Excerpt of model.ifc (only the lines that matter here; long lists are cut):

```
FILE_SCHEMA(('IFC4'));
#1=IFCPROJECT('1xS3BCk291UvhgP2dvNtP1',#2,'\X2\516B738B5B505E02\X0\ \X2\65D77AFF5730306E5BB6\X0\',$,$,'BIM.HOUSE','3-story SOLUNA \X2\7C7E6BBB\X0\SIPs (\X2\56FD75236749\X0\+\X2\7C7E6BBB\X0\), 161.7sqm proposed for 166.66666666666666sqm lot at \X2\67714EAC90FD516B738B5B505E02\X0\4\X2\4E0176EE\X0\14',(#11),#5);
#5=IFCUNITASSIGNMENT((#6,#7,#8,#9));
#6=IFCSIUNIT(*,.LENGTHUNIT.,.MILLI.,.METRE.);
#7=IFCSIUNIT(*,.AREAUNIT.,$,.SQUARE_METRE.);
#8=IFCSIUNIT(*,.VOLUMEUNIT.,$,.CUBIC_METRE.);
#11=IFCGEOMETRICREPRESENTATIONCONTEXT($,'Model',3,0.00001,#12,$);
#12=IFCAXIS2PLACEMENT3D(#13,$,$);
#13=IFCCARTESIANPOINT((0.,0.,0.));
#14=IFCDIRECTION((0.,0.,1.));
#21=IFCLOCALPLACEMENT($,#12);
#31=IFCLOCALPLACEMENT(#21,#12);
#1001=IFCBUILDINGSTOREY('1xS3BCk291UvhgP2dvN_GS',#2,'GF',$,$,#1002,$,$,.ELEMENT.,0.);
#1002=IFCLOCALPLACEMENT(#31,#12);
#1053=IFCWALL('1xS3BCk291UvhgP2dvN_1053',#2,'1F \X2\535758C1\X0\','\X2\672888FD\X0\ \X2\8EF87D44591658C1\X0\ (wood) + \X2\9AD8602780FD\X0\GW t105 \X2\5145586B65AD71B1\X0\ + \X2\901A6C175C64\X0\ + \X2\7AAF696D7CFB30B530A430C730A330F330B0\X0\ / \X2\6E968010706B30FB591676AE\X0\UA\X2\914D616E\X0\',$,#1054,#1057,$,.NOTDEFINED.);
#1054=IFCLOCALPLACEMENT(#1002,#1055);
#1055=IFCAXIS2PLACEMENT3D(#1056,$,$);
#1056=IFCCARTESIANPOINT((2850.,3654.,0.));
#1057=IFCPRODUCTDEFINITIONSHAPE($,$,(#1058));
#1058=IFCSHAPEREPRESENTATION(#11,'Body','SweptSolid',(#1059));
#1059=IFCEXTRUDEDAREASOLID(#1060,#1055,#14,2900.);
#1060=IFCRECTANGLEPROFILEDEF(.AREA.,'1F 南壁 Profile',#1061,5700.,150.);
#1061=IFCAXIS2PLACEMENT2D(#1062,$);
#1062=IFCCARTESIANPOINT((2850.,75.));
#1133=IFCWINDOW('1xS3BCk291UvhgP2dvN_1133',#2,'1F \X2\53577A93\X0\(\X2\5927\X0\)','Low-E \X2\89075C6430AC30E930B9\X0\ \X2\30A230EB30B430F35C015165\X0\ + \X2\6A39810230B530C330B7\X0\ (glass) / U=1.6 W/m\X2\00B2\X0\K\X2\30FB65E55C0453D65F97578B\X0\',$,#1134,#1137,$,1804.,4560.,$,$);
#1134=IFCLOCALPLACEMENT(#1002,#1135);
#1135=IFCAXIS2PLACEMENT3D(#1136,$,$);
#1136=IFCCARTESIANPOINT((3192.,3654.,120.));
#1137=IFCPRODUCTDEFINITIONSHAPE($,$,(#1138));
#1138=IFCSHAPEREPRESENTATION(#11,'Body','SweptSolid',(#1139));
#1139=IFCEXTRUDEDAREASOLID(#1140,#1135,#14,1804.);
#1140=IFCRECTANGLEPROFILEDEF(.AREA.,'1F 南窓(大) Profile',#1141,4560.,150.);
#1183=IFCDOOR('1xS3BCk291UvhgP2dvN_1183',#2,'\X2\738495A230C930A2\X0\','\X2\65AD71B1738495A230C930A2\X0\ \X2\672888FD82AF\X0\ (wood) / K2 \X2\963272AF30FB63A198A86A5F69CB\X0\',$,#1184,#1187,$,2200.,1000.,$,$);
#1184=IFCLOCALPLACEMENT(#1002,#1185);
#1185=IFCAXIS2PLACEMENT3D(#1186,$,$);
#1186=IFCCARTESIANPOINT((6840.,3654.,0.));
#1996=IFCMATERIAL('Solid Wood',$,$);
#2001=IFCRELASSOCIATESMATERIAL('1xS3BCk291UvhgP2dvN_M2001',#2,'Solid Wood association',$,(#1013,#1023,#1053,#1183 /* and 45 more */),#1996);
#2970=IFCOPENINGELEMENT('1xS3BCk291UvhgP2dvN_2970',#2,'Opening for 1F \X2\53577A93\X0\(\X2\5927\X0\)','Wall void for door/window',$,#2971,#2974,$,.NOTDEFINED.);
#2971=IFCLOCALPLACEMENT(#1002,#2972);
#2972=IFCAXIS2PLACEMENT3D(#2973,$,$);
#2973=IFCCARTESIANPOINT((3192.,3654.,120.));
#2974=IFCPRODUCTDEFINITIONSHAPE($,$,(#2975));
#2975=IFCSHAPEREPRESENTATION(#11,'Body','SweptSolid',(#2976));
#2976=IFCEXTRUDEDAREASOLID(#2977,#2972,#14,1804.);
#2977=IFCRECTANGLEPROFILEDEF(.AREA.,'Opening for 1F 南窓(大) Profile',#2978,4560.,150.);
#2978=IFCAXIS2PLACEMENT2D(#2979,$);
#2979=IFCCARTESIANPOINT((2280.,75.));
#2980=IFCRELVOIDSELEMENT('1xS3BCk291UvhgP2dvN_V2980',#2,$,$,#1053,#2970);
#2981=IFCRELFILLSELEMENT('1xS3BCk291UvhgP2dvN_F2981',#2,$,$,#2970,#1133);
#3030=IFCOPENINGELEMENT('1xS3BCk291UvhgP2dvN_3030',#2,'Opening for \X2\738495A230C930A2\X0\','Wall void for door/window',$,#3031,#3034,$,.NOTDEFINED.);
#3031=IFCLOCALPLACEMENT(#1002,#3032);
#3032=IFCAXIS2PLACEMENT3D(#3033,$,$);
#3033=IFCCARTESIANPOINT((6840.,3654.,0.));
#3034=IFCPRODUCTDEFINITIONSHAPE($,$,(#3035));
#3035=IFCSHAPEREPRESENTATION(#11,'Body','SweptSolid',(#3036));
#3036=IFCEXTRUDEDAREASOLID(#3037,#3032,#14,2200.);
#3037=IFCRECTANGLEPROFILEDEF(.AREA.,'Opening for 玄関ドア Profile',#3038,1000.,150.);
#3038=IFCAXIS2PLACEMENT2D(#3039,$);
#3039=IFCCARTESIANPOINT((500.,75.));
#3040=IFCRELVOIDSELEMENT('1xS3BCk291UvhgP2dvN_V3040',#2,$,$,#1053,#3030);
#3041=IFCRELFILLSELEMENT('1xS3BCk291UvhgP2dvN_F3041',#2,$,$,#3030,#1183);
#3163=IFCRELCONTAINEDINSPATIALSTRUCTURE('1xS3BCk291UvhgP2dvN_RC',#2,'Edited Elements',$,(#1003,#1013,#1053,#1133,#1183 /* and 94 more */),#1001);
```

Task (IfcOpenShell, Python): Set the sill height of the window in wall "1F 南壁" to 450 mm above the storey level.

```python
import numpy as np
import ifcopenshell
import ifcopenshell.api.geometry
import ifcopenshell.geom
import ifcopenshell.util.element
import ifcopenshell.util.placement
import ifcopenshell.util.shape
import ifcopenshell.util.unit

model = ifcopenshell.open("model.ifc")
unit_scale = ifcopenshell.util.unit.calculate_unit_scale(model)

window = model.by_guid("1xS3BCk291UvhgP2dvN_1133")
opening = window.FillsVoids[0].RelatingOpeningElement
storey = ifcopenshell.util.element.get_container(window, ifc_class="IfcBuildingStorey")
level = ifcopenshell.util.placement.get_local_placement(storey.ObjectPlacement)[2, 3]

# The opening's origin need not be at the sill, so measure its lowest point.
shape = ifcopenshell.geom.create_shape(ifcopenshell.geom.settings(), opening)
bottom = ifcopenshell.util.shape.get_shape_bottom_elevation(shape, shape.geometry) / unit_scale
dz = level + 0.45 / unit_scale - bottom

shift = np.array([0.0, 0.0, dz])
# The window is not placed relative to its opening, so move both.
for product in (opening, window):
    matrix = ifcopenshell.util.placement.get_local_placement(product.ObjectPlacement)
    matrix[:3, 3] += shift
    ifcopenshell.api.geometry.edit_object_placement(model, product=product, matrix=matrix, is_si=False)

print(f"moved by {dz * unit_scale:+.3f} m")

model.write("model_updated.ifc")
```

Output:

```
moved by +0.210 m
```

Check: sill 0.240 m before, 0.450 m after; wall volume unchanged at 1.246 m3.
